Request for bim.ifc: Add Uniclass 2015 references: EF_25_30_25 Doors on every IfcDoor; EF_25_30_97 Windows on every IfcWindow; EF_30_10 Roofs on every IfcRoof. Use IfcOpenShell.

First a look at what the model holds.

```python
import ifcopenshell

model = ifcopenshell.open("bim.ifc")
print(model.schema)
print("classifications:", [c.Name for c in model.by_type("IfcClassification")])
for ifc_class in ("IfcDoor", "IfcRoof", "IfcStair", "IfcWall", "IfcWindow"):
    print(ifc_class, len(model.by_type(ifc_class)))
```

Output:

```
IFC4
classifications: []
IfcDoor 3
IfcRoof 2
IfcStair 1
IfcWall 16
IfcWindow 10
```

```python
import ifcopenshell
import ifcopenshell.api.classification

model = ifcopenshell.open("bim.ifc")

system = ifcopenshell.api.classification.add_classification(model, classification="Uniclass 2015")

codes = {
    "IfcDoor": ("EF_25_30_25", "Doors"),
    "IfcWindow": ("EF_25_30_97", "Windows"),
    "IfcRoof": ("EF_30_10", "Roofs"),
}
for ifc_class, (code, name) in codes.items():
    products = model.by_type(ifc_class)
    ifcopenshell.api.classification.add_reference(
        model, products=products, classification=system, identification=code, name=name
    )
    print(code, len(products))

model.write("bim_v2.ifc")
```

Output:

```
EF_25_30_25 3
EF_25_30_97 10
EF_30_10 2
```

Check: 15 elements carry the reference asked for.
